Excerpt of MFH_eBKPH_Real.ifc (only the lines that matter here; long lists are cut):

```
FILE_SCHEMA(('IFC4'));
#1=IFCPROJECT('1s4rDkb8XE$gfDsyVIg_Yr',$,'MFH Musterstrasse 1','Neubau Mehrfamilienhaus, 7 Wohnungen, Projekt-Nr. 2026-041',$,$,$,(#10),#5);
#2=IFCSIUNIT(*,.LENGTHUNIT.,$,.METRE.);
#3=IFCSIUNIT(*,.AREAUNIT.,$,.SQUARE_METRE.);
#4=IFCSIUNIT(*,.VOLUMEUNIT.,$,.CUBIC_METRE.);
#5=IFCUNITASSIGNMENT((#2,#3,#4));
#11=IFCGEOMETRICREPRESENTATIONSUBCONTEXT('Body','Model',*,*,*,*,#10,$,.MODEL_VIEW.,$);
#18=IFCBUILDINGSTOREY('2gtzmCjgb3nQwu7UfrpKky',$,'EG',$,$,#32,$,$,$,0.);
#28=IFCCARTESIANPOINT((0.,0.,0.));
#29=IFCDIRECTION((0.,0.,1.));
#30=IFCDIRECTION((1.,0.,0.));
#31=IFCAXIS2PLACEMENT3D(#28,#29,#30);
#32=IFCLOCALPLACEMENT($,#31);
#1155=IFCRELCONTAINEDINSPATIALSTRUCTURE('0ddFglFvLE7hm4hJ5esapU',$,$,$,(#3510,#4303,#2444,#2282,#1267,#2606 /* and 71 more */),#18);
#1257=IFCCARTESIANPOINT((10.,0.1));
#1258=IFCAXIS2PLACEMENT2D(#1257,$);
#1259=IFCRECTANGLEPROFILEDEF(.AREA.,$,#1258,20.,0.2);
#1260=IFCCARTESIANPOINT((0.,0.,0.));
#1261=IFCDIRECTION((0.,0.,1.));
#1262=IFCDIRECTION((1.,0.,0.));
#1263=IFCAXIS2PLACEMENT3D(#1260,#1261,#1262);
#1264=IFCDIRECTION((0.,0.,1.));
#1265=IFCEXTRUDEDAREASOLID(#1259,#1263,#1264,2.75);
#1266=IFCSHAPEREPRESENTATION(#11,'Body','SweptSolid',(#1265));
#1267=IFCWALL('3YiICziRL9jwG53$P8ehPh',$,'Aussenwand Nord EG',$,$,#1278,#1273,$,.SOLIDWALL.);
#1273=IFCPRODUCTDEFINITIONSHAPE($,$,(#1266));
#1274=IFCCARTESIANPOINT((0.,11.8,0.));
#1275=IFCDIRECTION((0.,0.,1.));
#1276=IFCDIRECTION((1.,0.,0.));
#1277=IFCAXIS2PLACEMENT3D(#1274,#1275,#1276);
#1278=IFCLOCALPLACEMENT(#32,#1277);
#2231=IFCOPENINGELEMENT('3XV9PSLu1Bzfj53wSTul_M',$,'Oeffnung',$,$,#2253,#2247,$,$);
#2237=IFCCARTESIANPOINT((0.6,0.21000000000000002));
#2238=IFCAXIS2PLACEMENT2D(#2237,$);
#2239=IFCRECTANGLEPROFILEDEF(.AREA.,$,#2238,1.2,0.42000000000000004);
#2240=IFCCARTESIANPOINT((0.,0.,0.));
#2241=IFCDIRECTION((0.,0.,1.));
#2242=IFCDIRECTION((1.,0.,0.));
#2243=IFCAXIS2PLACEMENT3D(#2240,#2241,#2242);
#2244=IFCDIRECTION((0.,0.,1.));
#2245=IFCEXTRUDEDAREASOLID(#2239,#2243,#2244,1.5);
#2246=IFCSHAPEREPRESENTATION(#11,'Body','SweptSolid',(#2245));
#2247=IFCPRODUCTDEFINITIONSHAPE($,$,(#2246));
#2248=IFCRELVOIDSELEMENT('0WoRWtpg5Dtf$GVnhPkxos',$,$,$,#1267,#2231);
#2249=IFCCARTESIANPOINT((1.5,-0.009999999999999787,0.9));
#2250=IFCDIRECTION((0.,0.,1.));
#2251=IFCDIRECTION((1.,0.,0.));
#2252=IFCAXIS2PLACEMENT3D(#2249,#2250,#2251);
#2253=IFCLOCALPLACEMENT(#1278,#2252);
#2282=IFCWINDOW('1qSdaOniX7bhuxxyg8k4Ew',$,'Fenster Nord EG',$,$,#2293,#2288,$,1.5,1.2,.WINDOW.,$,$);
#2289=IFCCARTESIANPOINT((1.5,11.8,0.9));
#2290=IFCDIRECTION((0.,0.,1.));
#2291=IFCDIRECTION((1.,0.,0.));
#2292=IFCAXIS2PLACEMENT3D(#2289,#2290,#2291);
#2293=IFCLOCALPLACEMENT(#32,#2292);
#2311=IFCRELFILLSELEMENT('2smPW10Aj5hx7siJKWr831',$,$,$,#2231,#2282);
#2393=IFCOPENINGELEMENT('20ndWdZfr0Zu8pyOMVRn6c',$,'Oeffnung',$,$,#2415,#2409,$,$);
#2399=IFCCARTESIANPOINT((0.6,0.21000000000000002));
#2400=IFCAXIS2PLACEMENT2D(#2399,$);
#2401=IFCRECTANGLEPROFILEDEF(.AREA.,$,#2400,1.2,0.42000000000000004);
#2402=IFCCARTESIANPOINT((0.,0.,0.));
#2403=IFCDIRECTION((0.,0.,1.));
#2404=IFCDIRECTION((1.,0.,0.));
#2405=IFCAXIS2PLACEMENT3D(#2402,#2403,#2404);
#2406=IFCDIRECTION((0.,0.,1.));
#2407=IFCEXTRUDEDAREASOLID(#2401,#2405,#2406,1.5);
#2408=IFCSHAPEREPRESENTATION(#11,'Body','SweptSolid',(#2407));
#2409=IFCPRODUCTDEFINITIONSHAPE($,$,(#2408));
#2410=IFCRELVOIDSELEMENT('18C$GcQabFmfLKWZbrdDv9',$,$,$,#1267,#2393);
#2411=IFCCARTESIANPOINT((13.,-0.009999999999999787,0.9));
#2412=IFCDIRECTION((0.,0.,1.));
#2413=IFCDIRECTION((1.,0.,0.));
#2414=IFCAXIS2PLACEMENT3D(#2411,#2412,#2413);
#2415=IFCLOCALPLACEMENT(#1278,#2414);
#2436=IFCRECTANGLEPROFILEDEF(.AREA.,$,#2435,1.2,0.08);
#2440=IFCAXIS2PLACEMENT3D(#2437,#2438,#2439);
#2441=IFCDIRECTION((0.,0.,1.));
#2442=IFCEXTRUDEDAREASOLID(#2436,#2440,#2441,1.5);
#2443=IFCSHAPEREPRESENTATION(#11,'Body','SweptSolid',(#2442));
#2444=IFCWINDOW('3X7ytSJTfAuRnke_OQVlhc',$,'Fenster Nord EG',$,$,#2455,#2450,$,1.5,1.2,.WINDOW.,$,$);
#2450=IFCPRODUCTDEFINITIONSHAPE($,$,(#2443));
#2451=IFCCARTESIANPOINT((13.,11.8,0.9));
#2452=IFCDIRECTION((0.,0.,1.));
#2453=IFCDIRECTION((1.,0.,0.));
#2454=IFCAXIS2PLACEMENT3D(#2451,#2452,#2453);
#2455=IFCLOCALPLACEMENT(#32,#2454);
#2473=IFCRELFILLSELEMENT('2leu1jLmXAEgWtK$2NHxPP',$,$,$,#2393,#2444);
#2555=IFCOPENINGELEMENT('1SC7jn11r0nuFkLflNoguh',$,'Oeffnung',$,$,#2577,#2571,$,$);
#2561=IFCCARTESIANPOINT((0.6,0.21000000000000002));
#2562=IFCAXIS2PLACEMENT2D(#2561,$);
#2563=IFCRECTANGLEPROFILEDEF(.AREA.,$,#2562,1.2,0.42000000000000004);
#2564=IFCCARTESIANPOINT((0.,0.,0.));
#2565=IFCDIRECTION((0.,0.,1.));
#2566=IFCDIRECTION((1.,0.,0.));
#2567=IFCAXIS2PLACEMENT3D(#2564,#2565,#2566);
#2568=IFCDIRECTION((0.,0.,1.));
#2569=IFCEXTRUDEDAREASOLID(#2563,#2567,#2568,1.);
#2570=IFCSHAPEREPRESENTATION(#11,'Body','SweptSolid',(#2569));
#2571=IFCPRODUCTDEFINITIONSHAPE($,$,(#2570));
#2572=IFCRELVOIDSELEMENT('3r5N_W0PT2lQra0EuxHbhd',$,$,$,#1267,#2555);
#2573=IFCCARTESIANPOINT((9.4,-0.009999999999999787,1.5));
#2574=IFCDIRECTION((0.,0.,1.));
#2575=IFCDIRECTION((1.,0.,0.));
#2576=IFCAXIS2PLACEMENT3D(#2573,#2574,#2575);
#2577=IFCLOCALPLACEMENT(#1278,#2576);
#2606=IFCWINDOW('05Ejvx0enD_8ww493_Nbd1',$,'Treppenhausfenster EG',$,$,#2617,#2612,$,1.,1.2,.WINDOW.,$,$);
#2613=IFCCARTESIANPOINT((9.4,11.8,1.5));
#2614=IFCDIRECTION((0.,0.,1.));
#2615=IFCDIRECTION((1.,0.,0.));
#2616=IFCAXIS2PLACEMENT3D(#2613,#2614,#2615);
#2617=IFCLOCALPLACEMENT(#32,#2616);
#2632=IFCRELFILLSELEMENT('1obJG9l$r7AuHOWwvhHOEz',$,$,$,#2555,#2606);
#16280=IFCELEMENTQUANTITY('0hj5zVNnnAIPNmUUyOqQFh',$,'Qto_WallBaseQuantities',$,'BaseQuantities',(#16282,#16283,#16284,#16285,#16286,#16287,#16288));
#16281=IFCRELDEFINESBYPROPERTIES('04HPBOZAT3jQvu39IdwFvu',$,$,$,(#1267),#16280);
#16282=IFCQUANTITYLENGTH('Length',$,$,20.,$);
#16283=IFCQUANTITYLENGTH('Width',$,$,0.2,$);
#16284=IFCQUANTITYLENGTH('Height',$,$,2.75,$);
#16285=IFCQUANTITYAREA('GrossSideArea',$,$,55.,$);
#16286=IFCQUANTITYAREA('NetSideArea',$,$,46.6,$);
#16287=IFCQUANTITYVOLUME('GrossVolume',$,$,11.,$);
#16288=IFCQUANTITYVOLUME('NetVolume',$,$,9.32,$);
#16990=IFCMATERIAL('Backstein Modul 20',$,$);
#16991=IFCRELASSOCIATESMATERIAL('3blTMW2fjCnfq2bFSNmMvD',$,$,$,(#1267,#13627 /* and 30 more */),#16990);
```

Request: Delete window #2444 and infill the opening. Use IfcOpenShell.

```python
import ifcopenshell
import ifcopenshell.api.feature
import ifcopenshell.api.pset
import ifcopenshell.api.root
import ifcopenshell.geom
import ifcopenshell.util.element
import ifcopenshell.util.shape
import ifcopenshell.util.unit

model = ifcopenshell.open("MFH_eBKPH_Real.ifc")
area_scale = ifcopenshell.util.unit.calculate_unit_scale(model, "AREAUNIT")
volume_scale = ifcopenshell.util.unit.calculate_unit_scale(model, "VOLUMEUNIT")
settings = ifcopenshell.geom.settings()


def volume(element):
    """Net volume in cubic metres, openings subtracted."""
    shape = ifcopenshell.geom.create_shape(settings, element)
    return ifcopenshell.util.shape.get_volume(shape.geometry)


window = model.by_guid("3X7ytSJTfAuRnke_OQVlhc")
opening = window.FillsVoids[0].RelatingOpeningElement
wall = opening.VoidsElements[0].RelatingBuildingElement
before = volume(wall)

ifcopenshell.api.root.remove_product(model, product=window)
ifcopenshell.api.feature.remove_feature(model, feature=opening)

after = volume(wall)
thickness = 0.2  # wall thickness in metres

# Update the wall's stored quantities.
qto = model.by_id(ifcopenshell.util.element.get_pset(wall, "Qto_WallBaseQuantities", should_inherit=False)["id"])
ifcopenshell.api.pset.edit_qto(model, qto=qto, properties={
    "NetSideArea": after / thickness / area_scale,
    "NetVolume": after / volume_scale,
})

print(f"wall volume {before:.3f} -> {after:.3f} m3")

model.write("MFH_eBKPH_Real_rev.ifc")
```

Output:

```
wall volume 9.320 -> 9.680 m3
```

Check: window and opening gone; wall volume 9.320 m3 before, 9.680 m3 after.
